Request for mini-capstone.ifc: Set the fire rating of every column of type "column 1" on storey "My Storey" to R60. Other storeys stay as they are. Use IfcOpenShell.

First a look at what the model holds.

```python
import ifcopenshell
import ifcopenshell.util.element

model = ifcopenshell.open("mini-capstone.ifc")
print(model.schema)
storey = next(s for s in model.by_type("IfcBuildingStorey") if s.Name == "My Storey")
columns = [e for e in ifcopenshell.util.element.get_decomposition(storey) if e.is_a("IfcColumn")]
seen = {}
for e in columns:
    element_type = ifcopenshell.util.element.get_type(e)
    key = (element_type.Name if element_type != e and element_type else None, ifcopenshell.util.element.get_pset(e, "Pset_ColumnCommon", "FireRating"))
    seen[key] = seen.get(key, 0) + 1
for (name, value), count in sorted(seen.items(), key=str):
    print(count, "x", name, "|", value)
```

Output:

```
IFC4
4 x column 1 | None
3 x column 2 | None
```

```python
import ifcopenshell
import ifcopenshell.api.pset
import ifcopenshell.util.element

model = ifcopenshell.open("mini-capstone.ifc")

storey = next(s for s in model.by_type("IfcBuildingStorey") if s.Name == "My Storey")
columns = [e for e in ifcopenshell.util.element.get_decomposition(storey) if e.is_a("IfcColumn")]

count = 0
for e in columns:
    element_type = ifcopenshell.util.element.get_type(e)
    if element_type in (None, e) or element_type.Name != "column 1":
        continue
    # add_pset returns the element's existing set when there is one.
    pset = ifcopenshell.api.pset.add_pset(model, product=e, name="Pset_ColumnCommon")
    ifcopenshell.api.pset.edit_pset(model, pset=pset, properties={"FireRating": "R60"})
    count += 1

print(count, "columns updated")

model.write("mini-capstone_rev.ifc")
```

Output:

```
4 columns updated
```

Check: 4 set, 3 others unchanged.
